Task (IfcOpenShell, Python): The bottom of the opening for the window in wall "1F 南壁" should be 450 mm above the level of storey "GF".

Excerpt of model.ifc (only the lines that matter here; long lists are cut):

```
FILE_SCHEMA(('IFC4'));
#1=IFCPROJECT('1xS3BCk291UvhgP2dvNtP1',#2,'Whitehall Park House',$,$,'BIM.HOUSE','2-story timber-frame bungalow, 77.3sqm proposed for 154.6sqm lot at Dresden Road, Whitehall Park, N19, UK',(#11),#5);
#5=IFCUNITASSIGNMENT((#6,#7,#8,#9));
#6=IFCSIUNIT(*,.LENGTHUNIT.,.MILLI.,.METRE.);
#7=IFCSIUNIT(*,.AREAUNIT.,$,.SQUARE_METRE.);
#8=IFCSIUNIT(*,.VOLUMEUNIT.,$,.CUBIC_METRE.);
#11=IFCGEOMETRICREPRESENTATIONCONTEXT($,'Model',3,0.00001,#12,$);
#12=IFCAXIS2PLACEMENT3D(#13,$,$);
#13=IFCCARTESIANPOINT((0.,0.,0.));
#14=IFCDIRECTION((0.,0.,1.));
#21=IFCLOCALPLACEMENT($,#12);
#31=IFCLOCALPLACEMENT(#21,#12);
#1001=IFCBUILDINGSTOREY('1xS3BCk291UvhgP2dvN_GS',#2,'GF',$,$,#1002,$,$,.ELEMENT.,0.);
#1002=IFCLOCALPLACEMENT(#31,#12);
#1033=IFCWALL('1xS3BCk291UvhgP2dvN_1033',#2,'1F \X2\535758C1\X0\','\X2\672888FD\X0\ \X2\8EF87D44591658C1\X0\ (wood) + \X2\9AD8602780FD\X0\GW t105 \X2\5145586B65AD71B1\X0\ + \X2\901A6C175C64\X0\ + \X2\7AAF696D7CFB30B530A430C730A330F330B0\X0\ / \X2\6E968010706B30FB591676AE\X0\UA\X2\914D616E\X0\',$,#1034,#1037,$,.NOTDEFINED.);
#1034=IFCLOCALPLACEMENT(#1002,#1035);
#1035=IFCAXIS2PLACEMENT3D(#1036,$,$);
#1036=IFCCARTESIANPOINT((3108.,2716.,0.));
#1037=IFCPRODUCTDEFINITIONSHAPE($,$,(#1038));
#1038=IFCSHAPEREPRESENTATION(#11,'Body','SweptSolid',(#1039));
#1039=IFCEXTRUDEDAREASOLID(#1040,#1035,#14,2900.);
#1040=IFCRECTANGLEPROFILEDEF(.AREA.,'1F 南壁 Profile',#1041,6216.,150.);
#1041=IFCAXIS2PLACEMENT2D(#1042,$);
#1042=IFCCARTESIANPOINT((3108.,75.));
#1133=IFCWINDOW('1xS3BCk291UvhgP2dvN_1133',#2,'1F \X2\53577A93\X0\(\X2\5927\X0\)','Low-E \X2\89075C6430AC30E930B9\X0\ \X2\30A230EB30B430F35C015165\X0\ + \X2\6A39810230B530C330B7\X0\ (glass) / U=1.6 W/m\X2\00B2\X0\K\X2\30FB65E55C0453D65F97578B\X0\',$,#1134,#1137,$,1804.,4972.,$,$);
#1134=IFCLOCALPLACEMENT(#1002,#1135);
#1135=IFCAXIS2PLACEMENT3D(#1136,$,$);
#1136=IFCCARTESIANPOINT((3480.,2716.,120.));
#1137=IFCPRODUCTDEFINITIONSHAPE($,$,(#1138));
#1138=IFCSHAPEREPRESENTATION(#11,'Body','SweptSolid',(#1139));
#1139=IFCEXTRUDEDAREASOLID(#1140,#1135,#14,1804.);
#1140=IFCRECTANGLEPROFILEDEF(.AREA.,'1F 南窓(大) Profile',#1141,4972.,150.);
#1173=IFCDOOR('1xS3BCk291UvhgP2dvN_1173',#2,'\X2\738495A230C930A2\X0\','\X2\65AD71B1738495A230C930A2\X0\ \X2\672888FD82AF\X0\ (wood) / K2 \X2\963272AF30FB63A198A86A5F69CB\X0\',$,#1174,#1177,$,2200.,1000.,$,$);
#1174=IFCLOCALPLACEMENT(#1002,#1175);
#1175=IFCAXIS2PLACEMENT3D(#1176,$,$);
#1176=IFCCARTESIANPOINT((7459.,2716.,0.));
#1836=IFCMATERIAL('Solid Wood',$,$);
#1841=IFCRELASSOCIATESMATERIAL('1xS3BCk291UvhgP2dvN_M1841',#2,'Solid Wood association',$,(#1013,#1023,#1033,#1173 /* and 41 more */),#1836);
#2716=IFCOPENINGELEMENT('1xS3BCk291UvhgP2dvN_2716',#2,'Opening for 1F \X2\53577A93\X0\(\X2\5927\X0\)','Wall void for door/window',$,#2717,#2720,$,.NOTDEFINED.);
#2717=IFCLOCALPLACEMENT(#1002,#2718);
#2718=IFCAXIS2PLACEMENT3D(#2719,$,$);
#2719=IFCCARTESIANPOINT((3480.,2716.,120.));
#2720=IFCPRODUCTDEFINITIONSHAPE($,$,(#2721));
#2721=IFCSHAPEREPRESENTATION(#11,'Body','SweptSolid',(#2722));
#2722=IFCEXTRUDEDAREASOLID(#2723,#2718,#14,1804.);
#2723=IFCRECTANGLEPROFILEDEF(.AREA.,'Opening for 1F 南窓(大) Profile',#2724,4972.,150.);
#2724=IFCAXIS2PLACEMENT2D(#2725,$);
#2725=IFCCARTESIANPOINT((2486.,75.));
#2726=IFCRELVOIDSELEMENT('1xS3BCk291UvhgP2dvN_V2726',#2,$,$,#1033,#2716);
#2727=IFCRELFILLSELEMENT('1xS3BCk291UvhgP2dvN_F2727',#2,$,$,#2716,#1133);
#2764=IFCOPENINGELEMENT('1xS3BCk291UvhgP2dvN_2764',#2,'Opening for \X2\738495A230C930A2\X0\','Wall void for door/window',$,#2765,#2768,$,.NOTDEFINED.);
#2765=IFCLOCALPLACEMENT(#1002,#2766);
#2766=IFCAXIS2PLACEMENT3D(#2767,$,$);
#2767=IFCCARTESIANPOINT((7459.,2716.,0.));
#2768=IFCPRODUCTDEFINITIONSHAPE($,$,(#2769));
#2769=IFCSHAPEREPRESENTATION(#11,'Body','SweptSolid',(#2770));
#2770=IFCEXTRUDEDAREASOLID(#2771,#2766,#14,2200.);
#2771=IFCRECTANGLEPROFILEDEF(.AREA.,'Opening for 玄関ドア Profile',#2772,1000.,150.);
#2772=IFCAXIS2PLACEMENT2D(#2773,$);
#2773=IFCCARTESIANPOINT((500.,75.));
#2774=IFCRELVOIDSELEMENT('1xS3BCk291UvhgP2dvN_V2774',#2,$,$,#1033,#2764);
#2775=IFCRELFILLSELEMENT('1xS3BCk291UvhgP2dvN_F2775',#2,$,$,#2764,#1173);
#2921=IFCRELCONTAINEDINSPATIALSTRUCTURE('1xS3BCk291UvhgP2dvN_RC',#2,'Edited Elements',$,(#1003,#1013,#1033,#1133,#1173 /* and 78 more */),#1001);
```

```python
import numpy as np
import ifcopenshell
import ifcopenshell.api.geometry
import ifcopenshell.geom
import ifcopenshell.util.element
import ifcopenshell.util.placement
import ifcopenshell.util.shape
import ifcopenshell.util.unit

model = ifcopenshell.open("model.ifc")
unit_scale = ifcopenshell.util.unit.calculate_unit_scale(model)

window = model.by_guid("1xS3BCk291UvhgP2dvN_1133")
opening = window.FillsVoids[0].RelatingOpeningElement
storey = ifcopenshell.util.element.get_container(window, ifc_class="IfcBuildingStorey")
level = ifcopenshell.util.placement.get_local_placement(storey.ObjectPlacement)[2, 3]

# The opening's origin need not be at the sill, so measure its lowest point.
shape = ifcopenshell.geom.create_shape(ifcopenshell.geom.settings(), opening)
bottom = ifcopenshell.util.shape.get_shape_bottom_elevation(shape, shape.geometry) / unit_scale
dz = level + 0.45 / unit_scale - bottom

shift = np.array([0.0, 0.0, dz])
# The window is not placed relative to its opening, so move both.
for product in (opening, window):
    matrix = ifcopenshell.util.placement.get_local_placement(product.ObjectPlacement)
    matrix[:3, 3] += shift
    ifcopenshell.api.geometry.edit_object_placement(model, product=product, matrix=matrix, is_si=False)

print(f"moved by {dz * unit_scale:+.3f} m")

model.write("model_edited.ifc")
```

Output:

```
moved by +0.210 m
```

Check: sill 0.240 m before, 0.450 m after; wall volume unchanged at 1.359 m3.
